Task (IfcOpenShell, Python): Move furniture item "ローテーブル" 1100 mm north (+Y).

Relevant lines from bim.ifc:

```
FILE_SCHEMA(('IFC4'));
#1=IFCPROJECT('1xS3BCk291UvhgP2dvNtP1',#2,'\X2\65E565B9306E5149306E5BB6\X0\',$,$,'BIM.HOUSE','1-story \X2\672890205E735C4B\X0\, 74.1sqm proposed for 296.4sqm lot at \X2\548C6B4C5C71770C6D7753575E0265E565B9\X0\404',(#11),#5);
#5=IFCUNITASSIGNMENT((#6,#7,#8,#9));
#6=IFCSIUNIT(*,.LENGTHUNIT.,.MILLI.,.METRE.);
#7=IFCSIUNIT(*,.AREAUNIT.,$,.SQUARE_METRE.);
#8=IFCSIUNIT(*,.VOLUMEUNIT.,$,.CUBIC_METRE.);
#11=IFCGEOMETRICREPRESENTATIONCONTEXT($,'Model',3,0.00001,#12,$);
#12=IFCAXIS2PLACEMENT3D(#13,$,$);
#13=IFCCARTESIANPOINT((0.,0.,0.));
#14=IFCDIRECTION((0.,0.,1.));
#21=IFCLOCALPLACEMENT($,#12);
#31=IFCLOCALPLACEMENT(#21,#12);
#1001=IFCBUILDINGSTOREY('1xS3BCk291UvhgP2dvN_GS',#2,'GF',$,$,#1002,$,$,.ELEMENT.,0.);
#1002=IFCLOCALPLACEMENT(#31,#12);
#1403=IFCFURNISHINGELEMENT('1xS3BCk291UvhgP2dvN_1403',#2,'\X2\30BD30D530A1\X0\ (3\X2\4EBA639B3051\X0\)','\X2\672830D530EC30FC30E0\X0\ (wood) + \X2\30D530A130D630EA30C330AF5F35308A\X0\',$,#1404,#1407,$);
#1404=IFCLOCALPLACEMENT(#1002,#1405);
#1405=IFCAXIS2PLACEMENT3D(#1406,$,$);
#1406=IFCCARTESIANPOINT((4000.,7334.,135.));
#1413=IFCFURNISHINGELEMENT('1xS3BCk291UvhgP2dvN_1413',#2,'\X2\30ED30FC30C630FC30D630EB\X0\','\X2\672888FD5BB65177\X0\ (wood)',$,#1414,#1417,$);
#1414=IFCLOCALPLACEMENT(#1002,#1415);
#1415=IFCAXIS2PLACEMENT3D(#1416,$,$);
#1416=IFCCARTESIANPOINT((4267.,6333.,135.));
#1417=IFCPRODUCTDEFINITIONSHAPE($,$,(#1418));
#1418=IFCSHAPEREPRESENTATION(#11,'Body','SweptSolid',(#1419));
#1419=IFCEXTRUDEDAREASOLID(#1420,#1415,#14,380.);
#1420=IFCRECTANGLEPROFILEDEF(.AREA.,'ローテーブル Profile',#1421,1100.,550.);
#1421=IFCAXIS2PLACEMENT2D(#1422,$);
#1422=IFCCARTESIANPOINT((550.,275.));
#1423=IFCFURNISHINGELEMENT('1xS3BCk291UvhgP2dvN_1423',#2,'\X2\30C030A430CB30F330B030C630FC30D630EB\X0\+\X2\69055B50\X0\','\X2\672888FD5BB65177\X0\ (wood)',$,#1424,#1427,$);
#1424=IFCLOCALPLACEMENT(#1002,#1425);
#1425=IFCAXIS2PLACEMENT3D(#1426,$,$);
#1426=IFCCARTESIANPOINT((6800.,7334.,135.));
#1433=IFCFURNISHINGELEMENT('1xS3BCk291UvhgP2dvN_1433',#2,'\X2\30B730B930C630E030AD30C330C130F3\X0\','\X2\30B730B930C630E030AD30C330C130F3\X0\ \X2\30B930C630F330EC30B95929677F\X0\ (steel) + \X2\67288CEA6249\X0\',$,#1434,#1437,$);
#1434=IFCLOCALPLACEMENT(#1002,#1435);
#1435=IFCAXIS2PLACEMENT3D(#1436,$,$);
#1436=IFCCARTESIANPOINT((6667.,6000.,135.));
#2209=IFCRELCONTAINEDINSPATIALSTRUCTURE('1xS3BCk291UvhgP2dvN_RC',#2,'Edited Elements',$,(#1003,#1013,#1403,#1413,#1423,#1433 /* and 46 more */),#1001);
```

```python
import ifcopenshell
import ifcopenshell.api.geometry
import ifcopenshell.util.placement
import ifcopenshell.util.unit

model = ifcopenshell.open("bim.ifc")
unit_scale = ifcopenshell.util.unit.calculate_unit_scale(model)

item = model.by_guid("1xS3BCk291UvhgP2dvN_1413")
matrix = ifcopenshell.util.placement.get_local_placement(item.ObjectPlacement)
matrix[1, 3] += 1.1 / unit_scale
ifcopenshell.api.geometry.edit_object_placement(model, product=item, matrix=matrix, is_si=False)

print(ifcopenshell.util.placement.get_local_placement(item.ObjectPlacement).round(3) + 0.0)

model.write("bim_rev.ifc")
```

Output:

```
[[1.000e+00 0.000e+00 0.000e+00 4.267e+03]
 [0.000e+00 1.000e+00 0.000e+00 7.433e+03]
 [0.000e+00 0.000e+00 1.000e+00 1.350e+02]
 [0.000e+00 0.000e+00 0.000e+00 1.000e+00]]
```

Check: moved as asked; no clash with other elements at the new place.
